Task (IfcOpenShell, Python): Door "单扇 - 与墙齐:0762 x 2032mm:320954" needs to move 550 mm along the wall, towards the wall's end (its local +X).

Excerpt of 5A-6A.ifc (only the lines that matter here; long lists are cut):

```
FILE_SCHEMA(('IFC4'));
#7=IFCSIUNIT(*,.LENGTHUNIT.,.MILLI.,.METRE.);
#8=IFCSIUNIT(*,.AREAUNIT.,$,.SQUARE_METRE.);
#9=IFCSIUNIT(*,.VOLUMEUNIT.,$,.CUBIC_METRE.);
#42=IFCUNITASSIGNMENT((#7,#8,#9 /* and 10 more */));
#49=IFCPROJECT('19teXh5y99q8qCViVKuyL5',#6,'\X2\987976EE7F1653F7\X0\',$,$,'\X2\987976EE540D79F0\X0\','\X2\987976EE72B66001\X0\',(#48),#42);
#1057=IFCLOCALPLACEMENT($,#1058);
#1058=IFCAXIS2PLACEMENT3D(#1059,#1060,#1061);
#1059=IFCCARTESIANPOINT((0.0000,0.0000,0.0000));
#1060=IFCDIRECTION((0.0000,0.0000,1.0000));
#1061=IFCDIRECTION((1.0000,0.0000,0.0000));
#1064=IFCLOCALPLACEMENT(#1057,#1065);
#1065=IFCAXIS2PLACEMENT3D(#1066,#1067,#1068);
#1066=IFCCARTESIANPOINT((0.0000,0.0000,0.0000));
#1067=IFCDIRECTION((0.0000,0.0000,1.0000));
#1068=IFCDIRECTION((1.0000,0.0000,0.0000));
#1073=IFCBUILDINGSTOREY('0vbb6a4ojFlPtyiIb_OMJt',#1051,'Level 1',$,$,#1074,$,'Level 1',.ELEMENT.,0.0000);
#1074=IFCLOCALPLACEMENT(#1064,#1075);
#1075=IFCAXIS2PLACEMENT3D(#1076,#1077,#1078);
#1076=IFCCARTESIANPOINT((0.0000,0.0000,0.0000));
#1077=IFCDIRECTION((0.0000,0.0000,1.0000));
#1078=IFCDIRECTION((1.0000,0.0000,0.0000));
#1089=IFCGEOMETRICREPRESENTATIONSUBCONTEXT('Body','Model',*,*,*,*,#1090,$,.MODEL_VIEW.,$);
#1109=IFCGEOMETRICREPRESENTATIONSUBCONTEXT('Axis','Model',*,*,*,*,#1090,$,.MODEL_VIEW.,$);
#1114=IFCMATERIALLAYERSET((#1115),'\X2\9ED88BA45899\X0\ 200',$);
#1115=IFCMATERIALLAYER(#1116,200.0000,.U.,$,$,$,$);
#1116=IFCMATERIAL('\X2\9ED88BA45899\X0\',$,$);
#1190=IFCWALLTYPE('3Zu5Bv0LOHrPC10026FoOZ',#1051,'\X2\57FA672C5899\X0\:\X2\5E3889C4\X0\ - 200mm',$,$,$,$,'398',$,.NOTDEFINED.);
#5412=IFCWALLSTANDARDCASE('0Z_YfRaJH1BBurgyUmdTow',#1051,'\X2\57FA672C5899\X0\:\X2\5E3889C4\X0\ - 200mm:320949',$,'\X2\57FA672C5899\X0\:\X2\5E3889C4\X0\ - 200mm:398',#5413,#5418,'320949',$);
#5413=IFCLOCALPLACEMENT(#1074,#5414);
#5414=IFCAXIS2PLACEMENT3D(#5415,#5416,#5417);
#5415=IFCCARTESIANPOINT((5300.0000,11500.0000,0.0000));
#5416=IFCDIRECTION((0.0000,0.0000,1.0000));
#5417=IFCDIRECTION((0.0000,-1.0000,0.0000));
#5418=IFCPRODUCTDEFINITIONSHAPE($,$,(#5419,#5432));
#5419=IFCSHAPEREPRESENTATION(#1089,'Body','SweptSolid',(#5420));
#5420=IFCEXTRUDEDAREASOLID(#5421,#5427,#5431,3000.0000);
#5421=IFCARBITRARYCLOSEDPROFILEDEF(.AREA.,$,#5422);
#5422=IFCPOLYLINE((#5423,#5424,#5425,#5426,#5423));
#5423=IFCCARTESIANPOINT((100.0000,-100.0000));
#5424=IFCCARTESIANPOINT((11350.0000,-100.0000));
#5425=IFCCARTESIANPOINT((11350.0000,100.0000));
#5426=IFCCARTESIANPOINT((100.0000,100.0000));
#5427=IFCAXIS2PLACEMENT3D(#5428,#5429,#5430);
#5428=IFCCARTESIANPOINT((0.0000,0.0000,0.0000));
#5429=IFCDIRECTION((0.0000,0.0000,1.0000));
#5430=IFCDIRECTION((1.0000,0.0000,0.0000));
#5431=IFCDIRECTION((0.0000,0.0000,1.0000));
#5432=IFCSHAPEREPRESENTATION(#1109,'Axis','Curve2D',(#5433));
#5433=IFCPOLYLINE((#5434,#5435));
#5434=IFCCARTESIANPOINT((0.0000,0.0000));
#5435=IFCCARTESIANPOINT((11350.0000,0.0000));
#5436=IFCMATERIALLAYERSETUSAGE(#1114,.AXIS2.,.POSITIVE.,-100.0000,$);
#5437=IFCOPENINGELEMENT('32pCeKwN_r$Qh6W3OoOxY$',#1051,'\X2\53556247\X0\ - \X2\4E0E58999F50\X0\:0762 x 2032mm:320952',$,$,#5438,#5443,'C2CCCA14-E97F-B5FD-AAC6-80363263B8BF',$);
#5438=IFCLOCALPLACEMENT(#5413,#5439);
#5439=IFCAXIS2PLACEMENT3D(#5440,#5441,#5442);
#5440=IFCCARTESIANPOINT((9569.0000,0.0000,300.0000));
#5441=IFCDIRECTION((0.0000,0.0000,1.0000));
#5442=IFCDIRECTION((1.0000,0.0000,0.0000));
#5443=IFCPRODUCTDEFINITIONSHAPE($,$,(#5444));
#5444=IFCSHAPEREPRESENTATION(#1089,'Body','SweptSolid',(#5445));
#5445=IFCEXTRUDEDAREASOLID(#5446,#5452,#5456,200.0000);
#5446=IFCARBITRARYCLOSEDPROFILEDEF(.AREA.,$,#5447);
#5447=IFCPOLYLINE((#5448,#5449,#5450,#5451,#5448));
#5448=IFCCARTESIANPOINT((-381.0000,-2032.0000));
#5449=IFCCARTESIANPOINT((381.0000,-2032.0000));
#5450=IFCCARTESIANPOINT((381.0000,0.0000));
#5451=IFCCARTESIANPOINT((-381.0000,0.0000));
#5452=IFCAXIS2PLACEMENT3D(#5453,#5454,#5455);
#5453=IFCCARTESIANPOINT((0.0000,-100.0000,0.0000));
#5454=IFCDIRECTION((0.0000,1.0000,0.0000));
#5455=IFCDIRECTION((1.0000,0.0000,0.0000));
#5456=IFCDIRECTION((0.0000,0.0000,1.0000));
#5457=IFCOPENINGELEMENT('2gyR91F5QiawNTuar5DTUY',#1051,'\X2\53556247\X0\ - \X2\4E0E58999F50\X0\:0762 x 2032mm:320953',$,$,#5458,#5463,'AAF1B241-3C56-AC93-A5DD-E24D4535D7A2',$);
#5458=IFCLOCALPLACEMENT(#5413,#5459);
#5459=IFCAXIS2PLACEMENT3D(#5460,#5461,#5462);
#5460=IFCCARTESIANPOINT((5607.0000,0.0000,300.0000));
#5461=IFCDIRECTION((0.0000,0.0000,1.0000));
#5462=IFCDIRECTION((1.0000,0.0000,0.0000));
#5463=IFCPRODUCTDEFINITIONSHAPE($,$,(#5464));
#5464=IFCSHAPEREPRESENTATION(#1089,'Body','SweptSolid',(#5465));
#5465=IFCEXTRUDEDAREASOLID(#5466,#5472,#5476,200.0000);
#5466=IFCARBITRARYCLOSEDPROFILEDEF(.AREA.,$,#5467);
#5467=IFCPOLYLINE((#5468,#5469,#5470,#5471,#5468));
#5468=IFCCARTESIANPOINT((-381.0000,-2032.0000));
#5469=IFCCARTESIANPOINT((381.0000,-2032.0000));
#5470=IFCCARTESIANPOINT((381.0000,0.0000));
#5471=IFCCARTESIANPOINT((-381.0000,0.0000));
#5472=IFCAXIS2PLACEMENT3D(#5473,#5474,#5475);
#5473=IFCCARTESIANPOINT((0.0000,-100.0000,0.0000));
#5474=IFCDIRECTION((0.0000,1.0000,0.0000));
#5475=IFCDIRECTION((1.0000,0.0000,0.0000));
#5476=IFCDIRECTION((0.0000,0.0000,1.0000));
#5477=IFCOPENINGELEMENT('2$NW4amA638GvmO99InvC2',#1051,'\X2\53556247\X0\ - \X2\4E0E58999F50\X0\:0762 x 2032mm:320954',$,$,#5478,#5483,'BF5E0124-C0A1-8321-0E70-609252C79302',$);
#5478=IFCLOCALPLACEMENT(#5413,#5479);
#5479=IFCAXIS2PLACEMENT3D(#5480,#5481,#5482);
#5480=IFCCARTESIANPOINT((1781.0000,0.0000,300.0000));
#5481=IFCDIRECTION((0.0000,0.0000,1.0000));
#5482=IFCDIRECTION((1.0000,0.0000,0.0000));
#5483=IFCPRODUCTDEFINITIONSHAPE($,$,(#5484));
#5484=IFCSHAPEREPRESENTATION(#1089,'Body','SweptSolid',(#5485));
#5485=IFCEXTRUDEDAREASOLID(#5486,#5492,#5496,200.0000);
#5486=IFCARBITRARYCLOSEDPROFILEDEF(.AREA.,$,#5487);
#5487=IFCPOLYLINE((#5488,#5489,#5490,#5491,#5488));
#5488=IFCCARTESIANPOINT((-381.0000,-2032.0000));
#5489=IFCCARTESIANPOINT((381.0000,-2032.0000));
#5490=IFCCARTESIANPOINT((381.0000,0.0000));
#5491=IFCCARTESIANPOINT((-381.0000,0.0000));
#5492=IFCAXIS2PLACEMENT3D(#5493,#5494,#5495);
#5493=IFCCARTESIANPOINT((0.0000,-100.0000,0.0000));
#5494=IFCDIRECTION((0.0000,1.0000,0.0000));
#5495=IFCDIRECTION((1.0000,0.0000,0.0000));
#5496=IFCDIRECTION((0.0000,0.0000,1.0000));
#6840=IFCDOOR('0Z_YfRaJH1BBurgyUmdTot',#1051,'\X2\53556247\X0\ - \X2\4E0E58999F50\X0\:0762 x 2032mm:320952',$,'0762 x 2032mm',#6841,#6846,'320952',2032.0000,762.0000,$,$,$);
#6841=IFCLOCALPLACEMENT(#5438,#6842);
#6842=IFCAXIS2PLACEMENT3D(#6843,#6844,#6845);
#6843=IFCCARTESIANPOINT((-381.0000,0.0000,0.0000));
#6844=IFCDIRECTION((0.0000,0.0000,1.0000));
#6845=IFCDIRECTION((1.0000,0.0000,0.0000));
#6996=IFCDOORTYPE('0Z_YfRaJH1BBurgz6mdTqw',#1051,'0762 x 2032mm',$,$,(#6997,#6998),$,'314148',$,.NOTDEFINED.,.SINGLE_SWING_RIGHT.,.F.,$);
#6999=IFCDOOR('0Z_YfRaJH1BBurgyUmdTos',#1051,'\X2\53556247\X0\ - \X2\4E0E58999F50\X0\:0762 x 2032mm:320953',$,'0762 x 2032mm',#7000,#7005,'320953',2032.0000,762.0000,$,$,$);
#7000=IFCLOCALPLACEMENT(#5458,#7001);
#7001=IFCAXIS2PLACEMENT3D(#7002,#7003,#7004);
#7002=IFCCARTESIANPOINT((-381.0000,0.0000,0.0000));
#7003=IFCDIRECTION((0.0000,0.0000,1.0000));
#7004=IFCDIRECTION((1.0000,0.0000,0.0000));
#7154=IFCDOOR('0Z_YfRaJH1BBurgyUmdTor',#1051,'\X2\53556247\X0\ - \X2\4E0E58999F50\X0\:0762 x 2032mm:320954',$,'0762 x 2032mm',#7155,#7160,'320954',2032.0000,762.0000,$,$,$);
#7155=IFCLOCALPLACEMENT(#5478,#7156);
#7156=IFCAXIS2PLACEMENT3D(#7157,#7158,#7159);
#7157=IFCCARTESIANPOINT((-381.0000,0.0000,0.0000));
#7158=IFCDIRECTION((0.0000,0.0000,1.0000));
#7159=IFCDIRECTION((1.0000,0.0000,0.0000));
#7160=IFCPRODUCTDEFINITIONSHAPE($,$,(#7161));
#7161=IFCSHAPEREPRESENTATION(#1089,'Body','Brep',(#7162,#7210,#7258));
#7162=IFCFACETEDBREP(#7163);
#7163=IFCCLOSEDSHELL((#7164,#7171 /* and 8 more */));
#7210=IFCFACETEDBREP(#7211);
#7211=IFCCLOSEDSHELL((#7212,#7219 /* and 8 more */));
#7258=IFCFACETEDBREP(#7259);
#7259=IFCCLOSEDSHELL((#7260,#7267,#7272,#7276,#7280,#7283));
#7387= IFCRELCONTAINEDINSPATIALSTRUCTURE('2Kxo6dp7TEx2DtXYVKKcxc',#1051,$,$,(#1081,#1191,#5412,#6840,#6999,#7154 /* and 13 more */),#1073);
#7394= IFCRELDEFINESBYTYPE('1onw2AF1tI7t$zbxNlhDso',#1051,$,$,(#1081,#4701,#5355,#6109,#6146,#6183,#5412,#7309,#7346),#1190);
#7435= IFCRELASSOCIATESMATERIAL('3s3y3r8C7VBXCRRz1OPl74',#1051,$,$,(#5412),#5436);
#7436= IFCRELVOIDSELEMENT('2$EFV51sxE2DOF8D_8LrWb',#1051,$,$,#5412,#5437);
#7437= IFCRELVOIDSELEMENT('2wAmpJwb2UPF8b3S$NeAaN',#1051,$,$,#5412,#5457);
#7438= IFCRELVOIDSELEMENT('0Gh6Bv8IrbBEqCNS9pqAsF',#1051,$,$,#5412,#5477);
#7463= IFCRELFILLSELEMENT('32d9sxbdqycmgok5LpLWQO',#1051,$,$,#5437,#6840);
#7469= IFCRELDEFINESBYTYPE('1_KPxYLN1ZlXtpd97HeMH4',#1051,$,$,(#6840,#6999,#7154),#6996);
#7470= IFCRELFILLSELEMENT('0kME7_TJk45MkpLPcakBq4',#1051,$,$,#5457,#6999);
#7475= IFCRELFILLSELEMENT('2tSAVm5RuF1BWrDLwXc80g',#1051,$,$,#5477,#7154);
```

```python
import ifcopenshell
import ifcopenshell.api.geometry
import ifcopenshell.util.placement

model = ifcopenshell.open("5A-6A.ifc")

door = model.by_guid("0Z_YfRaJH1BBurgyUmdTor")
opening = door.FillsVoids[0].RelatingOpeningElement
wall = opening.VoidsElements[0].RelatingBuildingElement

wall_matrix = ifcopenshell.util.placement.get_local_placement(wall.ObjectPlacement)
shift = wall_matrix[:3, 0] * 550.0
before = ifcopenshell.util.placement.get_local_placement(door.ObjectPlacement)[:3, 3].copy()

# The door is placed relative to its opening, so it follows when the opening moves.
matrix = ifcopenshell.util.placement.get_local_placement(opening.ObjectPlacement)
matrix[:3, 3] += shift
ifcopenshell.api.geometry.edit_object_placement(
    model, product=opening, matrix=matrix, is_si=False, should_transform_children=True
)

after = ifcopenshell.util.placement.get_local_placement(door.ObjectPlacement)[:3, 3]
print("door moved by", (after - before).round(3) + 0.0)

model.write("5A-6A_updated.ifc")
```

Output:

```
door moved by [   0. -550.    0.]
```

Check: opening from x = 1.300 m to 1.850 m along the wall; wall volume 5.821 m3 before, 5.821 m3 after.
